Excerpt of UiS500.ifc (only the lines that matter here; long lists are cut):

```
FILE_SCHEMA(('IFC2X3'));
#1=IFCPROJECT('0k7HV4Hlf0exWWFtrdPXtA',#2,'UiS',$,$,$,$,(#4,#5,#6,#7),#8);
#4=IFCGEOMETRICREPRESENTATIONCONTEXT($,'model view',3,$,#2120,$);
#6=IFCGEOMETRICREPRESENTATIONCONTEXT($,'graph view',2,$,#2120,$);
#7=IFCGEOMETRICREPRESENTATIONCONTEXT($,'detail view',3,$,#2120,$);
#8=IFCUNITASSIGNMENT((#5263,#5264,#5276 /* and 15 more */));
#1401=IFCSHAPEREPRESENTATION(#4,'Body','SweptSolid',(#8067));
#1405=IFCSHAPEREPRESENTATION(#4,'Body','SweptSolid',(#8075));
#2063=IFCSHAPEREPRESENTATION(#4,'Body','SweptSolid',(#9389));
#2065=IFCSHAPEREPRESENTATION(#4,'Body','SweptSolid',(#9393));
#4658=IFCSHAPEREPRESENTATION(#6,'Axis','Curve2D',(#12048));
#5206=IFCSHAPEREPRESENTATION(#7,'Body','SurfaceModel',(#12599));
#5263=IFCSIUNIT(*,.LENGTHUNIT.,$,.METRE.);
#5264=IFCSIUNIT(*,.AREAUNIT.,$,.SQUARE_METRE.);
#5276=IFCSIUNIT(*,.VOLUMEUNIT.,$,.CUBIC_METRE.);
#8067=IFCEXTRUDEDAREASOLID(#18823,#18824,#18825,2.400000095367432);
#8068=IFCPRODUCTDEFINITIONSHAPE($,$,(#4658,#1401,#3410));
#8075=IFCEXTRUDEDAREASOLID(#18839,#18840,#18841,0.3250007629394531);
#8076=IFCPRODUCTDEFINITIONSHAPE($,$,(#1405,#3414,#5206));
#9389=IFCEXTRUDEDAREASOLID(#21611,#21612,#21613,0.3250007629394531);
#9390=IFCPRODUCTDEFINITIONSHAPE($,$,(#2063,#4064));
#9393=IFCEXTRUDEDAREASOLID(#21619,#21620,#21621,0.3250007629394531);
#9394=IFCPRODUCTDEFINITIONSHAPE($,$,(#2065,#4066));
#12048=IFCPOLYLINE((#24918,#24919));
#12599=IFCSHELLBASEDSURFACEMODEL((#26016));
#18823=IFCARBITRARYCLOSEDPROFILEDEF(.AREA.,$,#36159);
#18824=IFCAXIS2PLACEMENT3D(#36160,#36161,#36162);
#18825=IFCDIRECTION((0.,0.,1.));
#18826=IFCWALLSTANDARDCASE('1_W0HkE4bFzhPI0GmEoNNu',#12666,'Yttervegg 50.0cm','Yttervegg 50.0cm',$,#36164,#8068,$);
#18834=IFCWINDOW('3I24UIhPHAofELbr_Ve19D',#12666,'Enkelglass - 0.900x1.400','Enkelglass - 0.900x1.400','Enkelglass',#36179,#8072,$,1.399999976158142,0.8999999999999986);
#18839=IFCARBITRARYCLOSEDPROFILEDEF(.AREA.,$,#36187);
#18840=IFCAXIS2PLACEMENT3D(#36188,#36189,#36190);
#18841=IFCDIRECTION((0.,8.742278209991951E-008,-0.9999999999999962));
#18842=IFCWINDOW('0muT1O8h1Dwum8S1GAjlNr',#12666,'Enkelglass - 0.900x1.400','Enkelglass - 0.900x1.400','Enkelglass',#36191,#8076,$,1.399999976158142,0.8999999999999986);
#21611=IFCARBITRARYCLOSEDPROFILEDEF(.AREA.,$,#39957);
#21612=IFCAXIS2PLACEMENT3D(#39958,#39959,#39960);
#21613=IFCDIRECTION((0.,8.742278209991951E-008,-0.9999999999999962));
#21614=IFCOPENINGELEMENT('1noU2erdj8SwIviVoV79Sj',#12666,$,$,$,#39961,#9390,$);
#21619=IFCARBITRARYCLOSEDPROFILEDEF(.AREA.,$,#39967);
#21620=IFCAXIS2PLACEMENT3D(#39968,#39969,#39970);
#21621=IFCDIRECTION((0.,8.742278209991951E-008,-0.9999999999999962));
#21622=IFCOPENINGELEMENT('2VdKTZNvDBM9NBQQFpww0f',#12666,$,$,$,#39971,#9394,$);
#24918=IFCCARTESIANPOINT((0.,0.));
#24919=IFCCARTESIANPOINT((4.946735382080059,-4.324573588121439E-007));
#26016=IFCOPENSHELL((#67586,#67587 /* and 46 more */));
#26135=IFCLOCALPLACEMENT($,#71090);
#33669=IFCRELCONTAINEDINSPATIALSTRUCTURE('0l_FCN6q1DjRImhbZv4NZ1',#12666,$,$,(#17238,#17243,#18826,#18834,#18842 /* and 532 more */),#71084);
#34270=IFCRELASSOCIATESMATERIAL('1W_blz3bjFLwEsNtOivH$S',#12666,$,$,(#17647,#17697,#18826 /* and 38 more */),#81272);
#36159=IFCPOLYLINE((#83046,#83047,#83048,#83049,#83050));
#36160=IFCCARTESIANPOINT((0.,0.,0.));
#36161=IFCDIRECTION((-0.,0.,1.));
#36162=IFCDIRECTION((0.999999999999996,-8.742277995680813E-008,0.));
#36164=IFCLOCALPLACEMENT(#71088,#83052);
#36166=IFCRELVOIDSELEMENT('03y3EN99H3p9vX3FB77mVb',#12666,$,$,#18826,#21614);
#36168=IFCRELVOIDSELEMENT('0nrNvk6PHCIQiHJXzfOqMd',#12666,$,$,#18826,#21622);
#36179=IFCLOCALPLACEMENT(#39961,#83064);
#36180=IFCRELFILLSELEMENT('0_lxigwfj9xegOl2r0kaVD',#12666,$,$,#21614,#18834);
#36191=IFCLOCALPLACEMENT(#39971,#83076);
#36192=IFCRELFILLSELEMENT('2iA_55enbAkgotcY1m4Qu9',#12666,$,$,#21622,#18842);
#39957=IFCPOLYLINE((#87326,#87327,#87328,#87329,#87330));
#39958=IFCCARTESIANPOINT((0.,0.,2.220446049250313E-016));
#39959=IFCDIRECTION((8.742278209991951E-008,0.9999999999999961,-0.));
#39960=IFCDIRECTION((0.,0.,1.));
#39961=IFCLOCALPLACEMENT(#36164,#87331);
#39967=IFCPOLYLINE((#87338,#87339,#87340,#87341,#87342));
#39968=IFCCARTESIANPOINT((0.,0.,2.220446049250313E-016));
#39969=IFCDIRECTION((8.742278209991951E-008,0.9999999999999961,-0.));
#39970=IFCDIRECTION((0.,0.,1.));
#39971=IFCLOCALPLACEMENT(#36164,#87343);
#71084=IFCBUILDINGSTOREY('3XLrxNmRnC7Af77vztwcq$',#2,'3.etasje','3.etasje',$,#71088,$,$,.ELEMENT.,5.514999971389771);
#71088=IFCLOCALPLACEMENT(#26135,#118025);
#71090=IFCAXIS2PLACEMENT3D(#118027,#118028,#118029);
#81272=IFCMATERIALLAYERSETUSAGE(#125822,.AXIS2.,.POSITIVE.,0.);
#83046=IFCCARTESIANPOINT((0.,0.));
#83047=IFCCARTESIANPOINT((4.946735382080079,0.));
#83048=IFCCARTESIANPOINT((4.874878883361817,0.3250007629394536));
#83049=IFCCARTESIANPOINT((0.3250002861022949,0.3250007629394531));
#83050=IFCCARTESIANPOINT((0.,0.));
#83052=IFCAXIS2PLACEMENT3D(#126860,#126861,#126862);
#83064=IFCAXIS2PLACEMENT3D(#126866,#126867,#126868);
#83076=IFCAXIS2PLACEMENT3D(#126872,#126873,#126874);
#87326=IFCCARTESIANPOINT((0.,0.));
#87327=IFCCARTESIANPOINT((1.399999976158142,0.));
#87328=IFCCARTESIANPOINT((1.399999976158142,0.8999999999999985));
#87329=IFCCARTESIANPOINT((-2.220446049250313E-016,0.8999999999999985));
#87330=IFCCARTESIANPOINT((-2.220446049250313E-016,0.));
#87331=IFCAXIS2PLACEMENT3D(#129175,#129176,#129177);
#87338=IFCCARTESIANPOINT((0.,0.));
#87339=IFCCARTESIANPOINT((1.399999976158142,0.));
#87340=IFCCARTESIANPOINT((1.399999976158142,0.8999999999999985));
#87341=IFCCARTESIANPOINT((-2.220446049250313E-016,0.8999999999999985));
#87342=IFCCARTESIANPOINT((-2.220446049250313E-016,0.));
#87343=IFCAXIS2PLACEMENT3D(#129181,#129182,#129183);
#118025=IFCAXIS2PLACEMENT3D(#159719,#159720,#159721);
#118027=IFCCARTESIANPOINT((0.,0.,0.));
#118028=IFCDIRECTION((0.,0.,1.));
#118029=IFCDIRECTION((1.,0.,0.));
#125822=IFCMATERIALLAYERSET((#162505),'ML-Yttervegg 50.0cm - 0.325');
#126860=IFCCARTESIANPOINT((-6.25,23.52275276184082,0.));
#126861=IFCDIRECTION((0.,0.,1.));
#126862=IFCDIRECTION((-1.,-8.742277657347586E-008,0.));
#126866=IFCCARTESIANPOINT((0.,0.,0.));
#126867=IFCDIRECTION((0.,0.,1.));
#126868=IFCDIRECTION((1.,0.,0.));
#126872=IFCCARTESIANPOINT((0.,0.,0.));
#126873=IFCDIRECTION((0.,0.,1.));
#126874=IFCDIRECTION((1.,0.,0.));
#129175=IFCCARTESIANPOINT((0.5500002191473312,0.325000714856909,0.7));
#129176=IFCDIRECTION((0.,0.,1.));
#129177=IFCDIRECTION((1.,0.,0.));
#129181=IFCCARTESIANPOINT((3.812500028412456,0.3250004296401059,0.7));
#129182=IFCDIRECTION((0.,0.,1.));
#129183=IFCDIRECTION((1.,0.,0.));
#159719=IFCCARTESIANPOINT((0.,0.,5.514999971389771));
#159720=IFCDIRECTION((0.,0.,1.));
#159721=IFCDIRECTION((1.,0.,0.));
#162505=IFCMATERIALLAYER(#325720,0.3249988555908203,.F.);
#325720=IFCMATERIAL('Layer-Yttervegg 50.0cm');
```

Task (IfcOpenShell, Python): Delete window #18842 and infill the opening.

```python
import ifcopenshell
import ifcopenshell.api.feature
import ifcopenshell.api.root
import ifcopenshell.geom
import ifcopenshell.util.shape

model = ifcopenshell.open("UiS500.ifc")
settings = ifcopenshell.geom.settings()


def volume(element):
    """Net volume in cubic metres, openings subtracted."""
    shape = ifcopenshell.geom.create_shape(settings, element)
    return ifcopenshell.util.shape.get_volume(shape.geometry)


window = model.by_guid("0muT1O8h1Dwum8S1GAjlNr")
opening = window.FillsVoids[0].RelatingOpeningElement
wall = opening.VoidsElements[0].RelatingBuildingElement
before = volume(wall)

ifcopenshell.api.root.remove_product(model, product=window)
ifcopenshell.api.feature.remove_feature(model, feature=opening)

after = volume(wall)

print(f"wall volume {before:.3f} -> {after:.3f} m3")

model.write("UiS500_rev.ifc")
```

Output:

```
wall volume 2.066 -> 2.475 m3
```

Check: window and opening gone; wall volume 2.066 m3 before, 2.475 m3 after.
